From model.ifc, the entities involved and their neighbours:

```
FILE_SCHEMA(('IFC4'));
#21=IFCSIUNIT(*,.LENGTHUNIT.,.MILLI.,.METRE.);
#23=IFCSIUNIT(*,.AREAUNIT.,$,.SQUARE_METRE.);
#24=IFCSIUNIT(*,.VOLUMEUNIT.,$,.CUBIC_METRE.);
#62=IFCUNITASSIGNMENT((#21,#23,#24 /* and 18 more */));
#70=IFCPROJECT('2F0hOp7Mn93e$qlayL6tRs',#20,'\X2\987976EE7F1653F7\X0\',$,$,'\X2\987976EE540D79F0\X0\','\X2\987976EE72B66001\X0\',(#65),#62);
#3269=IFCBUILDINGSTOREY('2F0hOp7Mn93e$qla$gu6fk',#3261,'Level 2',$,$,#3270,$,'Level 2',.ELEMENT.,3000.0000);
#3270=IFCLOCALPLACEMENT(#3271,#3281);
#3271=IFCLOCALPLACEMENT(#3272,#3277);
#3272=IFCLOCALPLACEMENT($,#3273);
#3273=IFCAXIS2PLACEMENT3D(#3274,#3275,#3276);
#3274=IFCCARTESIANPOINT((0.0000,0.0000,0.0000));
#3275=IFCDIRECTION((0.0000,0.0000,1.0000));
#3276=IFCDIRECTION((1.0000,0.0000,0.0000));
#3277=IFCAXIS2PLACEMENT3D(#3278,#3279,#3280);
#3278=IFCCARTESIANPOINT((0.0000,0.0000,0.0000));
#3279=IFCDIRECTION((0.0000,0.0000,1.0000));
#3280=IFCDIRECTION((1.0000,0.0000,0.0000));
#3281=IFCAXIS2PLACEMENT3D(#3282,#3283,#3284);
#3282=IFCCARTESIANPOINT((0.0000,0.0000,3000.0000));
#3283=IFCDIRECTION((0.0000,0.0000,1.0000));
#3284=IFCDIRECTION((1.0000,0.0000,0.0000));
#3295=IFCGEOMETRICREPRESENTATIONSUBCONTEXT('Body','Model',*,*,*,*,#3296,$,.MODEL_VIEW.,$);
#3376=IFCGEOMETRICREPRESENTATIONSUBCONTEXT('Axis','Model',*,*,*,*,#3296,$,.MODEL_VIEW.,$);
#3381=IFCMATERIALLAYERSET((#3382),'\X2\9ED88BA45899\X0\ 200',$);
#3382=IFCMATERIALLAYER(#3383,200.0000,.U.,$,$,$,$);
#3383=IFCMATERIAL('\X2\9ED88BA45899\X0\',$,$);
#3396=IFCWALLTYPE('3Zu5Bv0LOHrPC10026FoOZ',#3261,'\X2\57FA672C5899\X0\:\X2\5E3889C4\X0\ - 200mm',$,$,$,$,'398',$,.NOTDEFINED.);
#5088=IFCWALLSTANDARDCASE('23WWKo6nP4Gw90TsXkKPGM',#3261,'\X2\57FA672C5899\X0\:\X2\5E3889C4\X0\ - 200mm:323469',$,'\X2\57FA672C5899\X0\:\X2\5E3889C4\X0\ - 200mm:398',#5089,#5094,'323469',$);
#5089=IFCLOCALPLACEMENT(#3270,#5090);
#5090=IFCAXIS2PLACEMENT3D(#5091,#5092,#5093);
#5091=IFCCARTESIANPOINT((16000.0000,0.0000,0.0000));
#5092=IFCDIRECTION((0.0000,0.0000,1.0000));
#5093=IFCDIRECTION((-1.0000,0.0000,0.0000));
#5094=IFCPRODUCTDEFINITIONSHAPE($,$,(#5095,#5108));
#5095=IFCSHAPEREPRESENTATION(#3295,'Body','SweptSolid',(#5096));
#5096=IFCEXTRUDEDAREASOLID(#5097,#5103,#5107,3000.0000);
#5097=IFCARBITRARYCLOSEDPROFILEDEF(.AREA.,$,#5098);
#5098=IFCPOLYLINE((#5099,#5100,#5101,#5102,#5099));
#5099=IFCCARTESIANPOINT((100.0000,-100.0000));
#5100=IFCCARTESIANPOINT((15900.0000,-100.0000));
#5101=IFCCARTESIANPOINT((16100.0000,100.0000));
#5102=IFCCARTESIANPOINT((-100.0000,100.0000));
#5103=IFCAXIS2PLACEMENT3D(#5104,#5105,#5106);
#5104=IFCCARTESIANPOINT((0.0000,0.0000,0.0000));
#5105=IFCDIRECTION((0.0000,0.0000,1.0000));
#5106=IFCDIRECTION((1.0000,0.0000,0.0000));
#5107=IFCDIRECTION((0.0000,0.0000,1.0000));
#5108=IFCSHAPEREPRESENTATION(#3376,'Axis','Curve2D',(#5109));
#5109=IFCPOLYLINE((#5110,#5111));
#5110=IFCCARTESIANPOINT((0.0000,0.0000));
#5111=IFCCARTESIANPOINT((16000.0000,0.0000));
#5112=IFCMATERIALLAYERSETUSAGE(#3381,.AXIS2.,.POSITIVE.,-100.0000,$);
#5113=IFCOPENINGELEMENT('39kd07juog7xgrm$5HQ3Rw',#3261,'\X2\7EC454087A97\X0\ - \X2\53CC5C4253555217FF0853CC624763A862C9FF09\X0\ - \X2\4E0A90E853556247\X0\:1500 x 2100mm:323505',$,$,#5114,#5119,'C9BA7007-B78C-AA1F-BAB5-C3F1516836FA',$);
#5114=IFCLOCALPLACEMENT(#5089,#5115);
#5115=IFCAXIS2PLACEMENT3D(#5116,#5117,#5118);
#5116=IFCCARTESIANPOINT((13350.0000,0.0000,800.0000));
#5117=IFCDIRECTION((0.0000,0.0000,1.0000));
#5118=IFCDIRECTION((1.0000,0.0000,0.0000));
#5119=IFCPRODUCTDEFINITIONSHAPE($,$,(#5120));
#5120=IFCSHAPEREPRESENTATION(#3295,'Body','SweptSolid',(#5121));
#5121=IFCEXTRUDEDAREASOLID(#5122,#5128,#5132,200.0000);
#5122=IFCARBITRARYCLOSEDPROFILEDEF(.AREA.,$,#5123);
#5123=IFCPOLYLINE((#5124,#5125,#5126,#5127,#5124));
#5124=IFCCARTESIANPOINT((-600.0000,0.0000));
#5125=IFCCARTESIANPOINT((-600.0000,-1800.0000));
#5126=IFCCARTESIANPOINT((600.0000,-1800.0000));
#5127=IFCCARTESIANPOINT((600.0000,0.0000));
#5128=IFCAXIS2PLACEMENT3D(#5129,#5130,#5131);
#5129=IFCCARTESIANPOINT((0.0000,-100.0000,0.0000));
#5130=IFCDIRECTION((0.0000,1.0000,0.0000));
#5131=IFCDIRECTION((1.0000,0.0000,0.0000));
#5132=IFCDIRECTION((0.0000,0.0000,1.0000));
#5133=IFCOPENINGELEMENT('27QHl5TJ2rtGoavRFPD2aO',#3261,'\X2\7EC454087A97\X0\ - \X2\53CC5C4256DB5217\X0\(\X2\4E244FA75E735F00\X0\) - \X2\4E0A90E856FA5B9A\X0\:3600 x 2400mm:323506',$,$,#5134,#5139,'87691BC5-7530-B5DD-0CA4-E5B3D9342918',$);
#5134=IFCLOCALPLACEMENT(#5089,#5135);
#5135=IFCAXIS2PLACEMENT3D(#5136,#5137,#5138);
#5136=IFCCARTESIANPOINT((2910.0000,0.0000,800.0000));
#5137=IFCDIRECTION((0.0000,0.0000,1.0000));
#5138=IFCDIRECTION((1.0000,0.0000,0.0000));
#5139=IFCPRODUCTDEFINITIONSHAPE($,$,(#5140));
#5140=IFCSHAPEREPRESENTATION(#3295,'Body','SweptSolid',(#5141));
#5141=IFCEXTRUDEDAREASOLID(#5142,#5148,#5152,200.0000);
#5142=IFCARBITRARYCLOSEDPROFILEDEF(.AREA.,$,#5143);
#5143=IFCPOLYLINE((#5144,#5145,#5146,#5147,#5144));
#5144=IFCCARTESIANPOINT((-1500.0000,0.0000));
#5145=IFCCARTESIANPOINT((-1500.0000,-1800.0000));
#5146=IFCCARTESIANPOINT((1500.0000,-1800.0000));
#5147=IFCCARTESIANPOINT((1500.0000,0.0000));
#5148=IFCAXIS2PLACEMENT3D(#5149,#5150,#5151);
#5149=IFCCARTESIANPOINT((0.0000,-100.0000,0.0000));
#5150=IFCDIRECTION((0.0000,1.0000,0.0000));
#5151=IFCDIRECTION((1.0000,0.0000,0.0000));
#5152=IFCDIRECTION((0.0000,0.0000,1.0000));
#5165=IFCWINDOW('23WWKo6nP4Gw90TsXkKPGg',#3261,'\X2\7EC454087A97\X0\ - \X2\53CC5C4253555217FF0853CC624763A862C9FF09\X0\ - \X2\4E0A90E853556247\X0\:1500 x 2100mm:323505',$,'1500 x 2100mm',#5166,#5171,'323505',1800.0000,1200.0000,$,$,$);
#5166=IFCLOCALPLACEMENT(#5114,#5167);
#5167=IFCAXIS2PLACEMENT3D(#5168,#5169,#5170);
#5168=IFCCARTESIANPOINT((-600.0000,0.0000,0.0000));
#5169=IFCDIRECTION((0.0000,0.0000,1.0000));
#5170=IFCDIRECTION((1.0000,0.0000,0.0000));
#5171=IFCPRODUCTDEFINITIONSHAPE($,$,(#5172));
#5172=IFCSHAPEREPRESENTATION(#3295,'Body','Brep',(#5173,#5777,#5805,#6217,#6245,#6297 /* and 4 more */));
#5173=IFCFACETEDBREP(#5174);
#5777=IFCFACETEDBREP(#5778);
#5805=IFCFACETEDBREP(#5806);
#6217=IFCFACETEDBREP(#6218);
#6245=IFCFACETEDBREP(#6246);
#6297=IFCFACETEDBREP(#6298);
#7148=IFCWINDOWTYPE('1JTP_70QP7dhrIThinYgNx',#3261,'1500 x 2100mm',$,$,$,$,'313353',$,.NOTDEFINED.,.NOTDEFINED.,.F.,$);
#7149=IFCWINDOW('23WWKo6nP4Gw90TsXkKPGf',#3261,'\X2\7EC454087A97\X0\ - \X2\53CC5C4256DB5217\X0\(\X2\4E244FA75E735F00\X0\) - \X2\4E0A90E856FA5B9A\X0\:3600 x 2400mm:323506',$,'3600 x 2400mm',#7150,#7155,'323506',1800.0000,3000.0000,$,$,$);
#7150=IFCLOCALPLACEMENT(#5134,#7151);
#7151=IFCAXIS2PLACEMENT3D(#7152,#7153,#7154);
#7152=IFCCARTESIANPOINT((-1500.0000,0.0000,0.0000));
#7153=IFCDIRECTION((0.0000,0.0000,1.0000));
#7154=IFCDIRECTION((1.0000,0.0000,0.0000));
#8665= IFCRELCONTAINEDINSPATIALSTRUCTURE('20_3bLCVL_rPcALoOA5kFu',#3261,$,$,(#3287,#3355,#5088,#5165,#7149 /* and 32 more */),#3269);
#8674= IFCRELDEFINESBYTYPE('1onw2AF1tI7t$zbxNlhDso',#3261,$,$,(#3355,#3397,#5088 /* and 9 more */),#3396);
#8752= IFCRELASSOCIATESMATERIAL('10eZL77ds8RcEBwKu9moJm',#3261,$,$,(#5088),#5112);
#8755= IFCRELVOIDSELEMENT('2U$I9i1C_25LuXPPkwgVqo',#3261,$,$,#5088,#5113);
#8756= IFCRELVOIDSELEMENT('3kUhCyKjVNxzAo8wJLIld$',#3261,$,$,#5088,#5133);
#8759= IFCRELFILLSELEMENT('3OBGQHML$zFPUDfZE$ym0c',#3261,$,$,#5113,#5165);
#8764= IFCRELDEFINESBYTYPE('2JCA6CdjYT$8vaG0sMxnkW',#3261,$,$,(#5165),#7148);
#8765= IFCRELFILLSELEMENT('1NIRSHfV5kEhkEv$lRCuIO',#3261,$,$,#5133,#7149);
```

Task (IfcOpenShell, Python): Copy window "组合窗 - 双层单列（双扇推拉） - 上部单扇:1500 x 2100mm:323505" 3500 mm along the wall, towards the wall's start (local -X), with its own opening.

```python
import ifcopenshell
import ifcopenshell.api.feature
import ifcopenshell.api.geometry
import ifcopenshell.api.root
import ifcopenshell.geom
import ifcopenshell.util.element
import ifcopenshell.util.placement
import ifcopenshell.util.shape

model = ifcopenshell.open("model.ifc")
settings = ifcopenshell.geom.settings()


def volume(element):
    """Net volume in cubic metres, openings subtracted."""
    shape = ifcopenshell.geom.create_shape(settings, element)
    return ifcopenshell.util.shape.get_volume(shape.geometry)


def reuse_history(source, copy):
    """copy_class also copies each property set's owner history, people and application; keep the originals."""
    for rel in copy.IsDefinedBy:
        if rel.is_a("IfcRelDefinesByProperties") and (history := rel.RelatingPropertyDefinition.OwnerHistory):
            rel.RelatingPropertyDefinition.OwnerHistory = source.OwnerHistory
            ifcopenshell.util.element.remove_deep2(model, history)


window = model.by_guid("23WWKo6nP4Gw90TsXkKPGg")
opening = window.FillsVoids[0].RelatingOpeningElement
wall = opening.VoidsElements[0].RelatingBuildingElement
before = volume(wall)
shift = ifcopenshell.util.placement.get_local_placement(wall.ObjectPlacement)[:3, 0] * -3500.0

# copy_class copies the void relationship, type, container and properties, but no geometry.
new_opening = ifcopenshell.api.root.copy_class(model, product=opening)
new_opening.Representation = ifcopenshell.util.element.copy_deep(
    model, opening.Representation, exclude=["IfcGeometricRepresentationContext", "IfcRepresentationMap"]
)
new_opening.Name = "组合窗 - 双层单列（双扇推拉） - 上部单扇:1500 x 2100mm"
new_opening.Tag = None
new_window = ifcopenshell.api.root.copy_class(model, product=window)
new_window.Representation = ifcopenshell.util.element.copy_deep(
    model, window.Representation, exclude=["IfcGeometricRepresentationContext", "IfcRepresentationMap"]
)
new_window.Name = "组合窗 - 双层单列（双扇推拉） - 上部单扇:1500 x 2100mm"
new_window.Tag = None
reuse_history(window, new_window)
ifcopenshell.api.feature.add_filling(model, opening=new_opening, element=new_window)

for old, new in ((opening, new_opening), (window, new_window)):
    matrix = ifcopenshell.util.placement.get_local_placement(old.ObjectPlacement)
    matrix[:3, 3] += shift
    ifcopenshell.api.geometry.edit_object_placement(model, product=new, matrix=matrix, is_si=False)

after = volume(wall)

print(f"wall volume {before:.3f} -> {after:.3f} m3")

model.write("model_edited.ifc")
```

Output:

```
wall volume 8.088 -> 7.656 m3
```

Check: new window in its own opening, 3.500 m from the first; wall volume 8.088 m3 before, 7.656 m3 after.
